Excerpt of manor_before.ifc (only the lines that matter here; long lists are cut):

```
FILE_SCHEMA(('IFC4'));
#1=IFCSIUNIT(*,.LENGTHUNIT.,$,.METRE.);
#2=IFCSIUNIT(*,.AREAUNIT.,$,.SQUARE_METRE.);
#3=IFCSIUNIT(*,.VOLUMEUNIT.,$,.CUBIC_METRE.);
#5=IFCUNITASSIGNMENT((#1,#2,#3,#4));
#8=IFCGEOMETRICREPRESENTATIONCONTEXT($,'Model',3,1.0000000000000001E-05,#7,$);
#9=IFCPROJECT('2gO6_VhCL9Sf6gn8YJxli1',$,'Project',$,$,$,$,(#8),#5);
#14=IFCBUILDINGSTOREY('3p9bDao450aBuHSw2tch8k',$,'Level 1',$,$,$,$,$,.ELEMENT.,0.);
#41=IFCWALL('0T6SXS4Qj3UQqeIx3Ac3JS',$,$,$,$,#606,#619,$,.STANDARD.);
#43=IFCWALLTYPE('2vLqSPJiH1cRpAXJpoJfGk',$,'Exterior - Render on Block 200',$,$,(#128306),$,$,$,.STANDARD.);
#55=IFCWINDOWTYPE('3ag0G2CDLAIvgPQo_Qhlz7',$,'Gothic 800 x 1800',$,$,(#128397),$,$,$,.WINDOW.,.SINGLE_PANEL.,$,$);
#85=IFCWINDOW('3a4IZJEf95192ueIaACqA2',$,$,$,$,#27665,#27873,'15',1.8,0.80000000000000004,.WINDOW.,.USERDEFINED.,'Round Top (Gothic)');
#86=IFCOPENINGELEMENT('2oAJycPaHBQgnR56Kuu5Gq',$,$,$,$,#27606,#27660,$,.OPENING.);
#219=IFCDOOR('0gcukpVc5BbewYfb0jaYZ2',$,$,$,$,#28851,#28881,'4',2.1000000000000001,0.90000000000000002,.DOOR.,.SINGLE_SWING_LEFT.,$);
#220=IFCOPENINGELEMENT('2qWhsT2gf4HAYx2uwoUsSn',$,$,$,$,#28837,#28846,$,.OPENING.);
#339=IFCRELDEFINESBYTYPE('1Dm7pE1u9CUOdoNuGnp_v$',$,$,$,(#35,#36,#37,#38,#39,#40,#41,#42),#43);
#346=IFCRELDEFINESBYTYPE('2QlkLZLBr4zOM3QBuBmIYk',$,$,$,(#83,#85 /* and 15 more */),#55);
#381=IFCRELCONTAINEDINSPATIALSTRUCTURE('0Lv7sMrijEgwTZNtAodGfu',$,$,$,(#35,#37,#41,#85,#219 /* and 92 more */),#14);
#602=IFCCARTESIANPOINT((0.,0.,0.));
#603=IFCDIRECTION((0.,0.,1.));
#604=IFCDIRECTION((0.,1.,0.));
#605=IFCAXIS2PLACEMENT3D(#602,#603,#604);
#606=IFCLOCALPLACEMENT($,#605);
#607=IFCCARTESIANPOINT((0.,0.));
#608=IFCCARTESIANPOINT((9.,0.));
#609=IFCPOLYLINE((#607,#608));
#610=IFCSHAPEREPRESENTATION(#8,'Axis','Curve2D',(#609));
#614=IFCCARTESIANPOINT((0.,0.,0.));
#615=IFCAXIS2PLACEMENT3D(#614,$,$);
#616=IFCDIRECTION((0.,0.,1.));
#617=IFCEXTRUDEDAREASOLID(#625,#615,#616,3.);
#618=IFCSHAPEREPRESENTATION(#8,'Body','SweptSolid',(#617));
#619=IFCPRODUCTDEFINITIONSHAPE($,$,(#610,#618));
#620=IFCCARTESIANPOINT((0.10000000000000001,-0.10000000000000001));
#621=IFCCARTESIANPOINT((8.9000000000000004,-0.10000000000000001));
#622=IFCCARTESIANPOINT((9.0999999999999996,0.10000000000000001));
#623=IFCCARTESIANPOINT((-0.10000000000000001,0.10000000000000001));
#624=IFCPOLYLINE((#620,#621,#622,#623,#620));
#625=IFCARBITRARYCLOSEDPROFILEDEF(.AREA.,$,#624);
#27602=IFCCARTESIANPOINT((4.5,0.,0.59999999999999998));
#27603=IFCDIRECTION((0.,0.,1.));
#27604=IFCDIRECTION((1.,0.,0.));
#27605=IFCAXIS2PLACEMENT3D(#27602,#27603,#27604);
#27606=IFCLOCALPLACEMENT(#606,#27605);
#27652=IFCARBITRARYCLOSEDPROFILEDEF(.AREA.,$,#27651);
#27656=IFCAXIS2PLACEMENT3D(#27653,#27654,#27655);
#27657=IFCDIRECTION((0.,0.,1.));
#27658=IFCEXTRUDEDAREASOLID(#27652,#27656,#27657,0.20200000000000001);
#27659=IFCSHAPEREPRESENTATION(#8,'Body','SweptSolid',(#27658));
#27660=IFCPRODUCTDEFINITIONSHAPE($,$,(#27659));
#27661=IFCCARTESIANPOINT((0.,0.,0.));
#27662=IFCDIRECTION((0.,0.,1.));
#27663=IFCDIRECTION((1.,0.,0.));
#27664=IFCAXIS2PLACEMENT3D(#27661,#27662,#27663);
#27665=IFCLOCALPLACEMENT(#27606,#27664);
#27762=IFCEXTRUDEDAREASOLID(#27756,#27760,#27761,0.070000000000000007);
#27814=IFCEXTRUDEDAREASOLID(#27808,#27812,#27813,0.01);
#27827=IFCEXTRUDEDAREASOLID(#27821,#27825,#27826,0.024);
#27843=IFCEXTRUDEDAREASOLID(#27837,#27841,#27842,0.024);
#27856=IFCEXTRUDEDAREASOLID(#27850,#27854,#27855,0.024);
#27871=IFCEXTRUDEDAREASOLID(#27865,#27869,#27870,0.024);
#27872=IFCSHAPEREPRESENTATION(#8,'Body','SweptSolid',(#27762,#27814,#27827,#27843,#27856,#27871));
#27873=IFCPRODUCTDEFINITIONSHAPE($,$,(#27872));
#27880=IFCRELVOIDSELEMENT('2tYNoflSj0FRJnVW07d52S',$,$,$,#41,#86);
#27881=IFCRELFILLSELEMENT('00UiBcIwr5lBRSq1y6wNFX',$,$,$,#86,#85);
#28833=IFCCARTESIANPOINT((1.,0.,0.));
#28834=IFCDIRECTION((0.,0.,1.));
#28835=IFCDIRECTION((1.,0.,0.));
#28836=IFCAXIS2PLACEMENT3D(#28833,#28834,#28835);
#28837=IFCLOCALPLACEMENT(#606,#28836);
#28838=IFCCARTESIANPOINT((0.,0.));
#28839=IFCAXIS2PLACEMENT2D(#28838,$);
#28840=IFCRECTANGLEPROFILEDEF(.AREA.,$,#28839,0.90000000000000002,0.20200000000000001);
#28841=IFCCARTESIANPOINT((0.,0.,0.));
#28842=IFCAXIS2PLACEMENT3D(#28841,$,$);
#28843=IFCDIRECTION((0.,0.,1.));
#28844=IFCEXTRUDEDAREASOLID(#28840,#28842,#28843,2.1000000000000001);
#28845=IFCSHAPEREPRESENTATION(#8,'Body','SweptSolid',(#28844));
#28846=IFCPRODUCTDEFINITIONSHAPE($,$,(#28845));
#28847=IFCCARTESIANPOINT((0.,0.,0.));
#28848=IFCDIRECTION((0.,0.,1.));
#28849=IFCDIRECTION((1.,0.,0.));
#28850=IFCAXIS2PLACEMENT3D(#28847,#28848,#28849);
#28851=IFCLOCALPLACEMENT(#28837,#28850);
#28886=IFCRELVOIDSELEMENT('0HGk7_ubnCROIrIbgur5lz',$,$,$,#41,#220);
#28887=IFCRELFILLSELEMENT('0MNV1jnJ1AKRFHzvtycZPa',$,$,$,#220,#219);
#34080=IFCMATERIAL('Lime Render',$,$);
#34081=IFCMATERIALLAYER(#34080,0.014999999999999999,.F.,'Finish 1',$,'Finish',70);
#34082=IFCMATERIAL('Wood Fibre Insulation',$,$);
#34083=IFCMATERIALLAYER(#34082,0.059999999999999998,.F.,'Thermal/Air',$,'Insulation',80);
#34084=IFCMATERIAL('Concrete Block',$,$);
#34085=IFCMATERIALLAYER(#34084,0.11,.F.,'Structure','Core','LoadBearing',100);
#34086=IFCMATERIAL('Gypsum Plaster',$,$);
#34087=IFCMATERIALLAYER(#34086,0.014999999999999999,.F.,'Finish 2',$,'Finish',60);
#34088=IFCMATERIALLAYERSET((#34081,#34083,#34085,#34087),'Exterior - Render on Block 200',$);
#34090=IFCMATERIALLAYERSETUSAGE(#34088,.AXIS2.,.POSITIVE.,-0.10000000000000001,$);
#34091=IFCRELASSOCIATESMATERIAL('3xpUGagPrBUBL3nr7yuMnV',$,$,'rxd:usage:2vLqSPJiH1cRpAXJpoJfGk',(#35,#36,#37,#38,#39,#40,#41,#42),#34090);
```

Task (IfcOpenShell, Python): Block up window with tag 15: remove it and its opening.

```python
import ifcopenshell
import ifcopenshell.api.feature
import ifcopenshell.api.root
import ifcopenshell.geom
import ifcopenshell.util.shape

model = ifcopenshell.open("manor_before.ifc")
settings = ifcopenshell.geom.settings()


def volume(element):
    """Net volume in cubic metres, openings subtracted."""
    shape = ifcopenshell.geom.create_shape(settings, element)
    return ifcopenshell.util.shape.get_volume(shape.geometry)


window = model.by_guid("3a4IZJEf95192ueIaACqA2")
opening = window.FillsVoids[0].RelatingOpeningElement
wall = opening.VoidsElements[0].RelatingBuildingElement
before = volume(wall)

ifcopenshell.api.root.remove_product(model, product=window)
ifcopenshell.api.feature.remove_feature(model, feature=opening)

after = volume(wall)

print(f"wall volume {before:.3f} -> {after:.3f} m3")

model.write("manor_before_edited.ifc")
```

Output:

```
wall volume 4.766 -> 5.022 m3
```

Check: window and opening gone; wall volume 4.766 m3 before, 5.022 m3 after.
